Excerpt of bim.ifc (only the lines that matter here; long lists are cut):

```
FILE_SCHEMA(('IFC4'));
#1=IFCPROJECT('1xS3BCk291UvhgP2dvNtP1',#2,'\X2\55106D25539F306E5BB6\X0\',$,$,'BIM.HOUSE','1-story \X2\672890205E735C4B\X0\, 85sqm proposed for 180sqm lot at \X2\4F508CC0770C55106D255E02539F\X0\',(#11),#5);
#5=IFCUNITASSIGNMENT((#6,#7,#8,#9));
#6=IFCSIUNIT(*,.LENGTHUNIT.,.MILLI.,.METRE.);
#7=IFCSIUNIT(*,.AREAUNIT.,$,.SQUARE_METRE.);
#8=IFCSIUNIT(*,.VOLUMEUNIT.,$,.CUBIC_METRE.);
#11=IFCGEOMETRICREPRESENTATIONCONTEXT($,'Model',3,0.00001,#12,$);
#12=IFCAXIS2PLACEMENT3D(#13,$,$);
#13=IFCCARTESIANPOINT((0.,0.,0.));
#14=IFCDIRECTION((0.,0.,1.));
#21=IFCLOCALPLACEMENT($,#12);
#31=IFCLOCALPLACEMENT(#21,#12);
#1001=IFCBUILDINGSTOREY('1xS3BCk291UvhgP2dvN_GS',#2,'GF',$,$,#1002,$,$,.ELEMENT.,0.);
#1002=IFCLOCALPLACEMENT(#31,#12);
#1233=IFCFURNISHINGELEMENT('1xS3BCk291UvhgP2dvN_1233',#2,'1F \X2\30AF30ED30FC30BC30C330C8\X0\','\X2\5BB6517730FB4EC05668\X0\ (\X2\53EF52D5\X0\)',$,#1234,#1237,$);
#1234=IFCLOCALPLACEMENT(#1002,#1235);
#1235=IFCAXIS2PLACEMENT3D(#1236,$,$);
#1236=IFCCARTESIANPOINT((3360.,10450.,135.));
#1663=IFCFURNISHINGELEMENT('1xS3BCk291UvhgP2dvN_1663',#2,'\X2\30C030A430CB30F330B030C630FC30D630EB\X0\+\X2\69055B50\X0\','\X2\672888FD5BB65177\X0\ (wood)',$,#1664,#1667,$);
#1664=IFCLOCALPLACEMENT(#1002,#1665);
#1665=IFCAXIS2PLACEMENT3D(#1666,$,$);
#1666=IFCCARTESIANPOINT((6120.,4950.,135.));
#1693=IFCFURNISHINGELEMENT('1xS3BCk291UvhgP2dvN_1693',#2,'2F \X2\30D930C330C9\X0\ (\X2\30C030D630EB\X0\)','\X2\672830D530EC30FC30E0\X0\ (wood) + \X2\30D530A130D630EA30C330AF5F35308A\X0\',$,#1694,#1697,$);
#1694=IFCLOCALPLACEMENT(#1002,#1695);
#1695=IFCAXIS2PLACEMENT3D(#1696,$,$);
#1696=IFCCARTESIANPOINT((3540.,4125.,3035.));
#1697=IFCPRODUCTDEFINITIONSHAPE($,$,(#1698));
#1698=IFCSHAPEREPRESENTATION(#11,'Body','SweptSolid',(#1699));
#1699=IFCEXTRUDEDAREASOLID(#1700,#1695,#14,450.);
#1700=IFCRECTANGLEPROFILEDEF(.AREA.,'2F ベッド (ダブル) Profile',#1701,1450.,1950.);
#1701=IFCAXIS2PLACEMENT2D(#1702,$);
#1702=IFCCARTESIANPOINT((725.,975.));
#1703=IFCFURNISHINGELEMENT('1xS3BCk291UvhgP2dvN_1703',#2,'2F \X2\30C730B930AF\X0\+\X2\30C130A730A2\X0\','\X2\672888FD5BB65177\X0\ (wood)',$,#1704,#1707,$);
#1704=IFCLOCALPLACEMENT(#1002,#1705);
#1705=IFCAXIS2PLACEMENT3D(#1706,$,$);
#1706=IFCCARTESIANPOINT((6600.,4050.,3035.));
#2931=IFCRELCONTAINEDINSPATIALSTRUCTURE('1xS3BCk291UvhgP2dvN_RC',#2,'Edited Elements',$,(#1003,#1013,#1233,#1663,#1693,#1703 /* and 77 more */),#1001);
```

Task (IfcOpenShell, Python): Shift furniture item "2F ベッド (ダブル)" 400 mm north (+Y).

```python
import ifcopenshell
import ifcopenshell.api.geometry
import ifcopenshell.util.placement
import ifcopenshell.util.unit

model = ifcopenshell.open("bim.ifc")
unit_scale = ifcopenshell.util.unit.calculate_unit_scale(model)

item = model.by_guid("1xS3BCk291UvhgP2dvN_1693")
matrix = ifcopenshell.util.placement.get_local_placement(item.ObjectPlacement)
matrix[1, 3] += 0.4 / unit_scale
ifcopenshell.api.geometry.edit_object_placement(model, product=item, matrix=matrix, is_si=False)

print(ifcopenshell.util.placement.get_local_placement(item.ObjectPlacement).round(3) + 0.0)

model.write("bim-out.ifc")
```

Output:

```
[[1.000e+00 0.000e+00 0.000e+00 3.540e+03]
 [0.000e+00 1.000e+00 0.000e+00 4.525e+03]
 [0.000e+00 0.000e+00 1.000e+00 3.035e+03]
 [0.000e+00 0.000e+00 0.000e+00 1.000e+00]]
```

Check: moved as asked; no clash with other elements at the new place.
